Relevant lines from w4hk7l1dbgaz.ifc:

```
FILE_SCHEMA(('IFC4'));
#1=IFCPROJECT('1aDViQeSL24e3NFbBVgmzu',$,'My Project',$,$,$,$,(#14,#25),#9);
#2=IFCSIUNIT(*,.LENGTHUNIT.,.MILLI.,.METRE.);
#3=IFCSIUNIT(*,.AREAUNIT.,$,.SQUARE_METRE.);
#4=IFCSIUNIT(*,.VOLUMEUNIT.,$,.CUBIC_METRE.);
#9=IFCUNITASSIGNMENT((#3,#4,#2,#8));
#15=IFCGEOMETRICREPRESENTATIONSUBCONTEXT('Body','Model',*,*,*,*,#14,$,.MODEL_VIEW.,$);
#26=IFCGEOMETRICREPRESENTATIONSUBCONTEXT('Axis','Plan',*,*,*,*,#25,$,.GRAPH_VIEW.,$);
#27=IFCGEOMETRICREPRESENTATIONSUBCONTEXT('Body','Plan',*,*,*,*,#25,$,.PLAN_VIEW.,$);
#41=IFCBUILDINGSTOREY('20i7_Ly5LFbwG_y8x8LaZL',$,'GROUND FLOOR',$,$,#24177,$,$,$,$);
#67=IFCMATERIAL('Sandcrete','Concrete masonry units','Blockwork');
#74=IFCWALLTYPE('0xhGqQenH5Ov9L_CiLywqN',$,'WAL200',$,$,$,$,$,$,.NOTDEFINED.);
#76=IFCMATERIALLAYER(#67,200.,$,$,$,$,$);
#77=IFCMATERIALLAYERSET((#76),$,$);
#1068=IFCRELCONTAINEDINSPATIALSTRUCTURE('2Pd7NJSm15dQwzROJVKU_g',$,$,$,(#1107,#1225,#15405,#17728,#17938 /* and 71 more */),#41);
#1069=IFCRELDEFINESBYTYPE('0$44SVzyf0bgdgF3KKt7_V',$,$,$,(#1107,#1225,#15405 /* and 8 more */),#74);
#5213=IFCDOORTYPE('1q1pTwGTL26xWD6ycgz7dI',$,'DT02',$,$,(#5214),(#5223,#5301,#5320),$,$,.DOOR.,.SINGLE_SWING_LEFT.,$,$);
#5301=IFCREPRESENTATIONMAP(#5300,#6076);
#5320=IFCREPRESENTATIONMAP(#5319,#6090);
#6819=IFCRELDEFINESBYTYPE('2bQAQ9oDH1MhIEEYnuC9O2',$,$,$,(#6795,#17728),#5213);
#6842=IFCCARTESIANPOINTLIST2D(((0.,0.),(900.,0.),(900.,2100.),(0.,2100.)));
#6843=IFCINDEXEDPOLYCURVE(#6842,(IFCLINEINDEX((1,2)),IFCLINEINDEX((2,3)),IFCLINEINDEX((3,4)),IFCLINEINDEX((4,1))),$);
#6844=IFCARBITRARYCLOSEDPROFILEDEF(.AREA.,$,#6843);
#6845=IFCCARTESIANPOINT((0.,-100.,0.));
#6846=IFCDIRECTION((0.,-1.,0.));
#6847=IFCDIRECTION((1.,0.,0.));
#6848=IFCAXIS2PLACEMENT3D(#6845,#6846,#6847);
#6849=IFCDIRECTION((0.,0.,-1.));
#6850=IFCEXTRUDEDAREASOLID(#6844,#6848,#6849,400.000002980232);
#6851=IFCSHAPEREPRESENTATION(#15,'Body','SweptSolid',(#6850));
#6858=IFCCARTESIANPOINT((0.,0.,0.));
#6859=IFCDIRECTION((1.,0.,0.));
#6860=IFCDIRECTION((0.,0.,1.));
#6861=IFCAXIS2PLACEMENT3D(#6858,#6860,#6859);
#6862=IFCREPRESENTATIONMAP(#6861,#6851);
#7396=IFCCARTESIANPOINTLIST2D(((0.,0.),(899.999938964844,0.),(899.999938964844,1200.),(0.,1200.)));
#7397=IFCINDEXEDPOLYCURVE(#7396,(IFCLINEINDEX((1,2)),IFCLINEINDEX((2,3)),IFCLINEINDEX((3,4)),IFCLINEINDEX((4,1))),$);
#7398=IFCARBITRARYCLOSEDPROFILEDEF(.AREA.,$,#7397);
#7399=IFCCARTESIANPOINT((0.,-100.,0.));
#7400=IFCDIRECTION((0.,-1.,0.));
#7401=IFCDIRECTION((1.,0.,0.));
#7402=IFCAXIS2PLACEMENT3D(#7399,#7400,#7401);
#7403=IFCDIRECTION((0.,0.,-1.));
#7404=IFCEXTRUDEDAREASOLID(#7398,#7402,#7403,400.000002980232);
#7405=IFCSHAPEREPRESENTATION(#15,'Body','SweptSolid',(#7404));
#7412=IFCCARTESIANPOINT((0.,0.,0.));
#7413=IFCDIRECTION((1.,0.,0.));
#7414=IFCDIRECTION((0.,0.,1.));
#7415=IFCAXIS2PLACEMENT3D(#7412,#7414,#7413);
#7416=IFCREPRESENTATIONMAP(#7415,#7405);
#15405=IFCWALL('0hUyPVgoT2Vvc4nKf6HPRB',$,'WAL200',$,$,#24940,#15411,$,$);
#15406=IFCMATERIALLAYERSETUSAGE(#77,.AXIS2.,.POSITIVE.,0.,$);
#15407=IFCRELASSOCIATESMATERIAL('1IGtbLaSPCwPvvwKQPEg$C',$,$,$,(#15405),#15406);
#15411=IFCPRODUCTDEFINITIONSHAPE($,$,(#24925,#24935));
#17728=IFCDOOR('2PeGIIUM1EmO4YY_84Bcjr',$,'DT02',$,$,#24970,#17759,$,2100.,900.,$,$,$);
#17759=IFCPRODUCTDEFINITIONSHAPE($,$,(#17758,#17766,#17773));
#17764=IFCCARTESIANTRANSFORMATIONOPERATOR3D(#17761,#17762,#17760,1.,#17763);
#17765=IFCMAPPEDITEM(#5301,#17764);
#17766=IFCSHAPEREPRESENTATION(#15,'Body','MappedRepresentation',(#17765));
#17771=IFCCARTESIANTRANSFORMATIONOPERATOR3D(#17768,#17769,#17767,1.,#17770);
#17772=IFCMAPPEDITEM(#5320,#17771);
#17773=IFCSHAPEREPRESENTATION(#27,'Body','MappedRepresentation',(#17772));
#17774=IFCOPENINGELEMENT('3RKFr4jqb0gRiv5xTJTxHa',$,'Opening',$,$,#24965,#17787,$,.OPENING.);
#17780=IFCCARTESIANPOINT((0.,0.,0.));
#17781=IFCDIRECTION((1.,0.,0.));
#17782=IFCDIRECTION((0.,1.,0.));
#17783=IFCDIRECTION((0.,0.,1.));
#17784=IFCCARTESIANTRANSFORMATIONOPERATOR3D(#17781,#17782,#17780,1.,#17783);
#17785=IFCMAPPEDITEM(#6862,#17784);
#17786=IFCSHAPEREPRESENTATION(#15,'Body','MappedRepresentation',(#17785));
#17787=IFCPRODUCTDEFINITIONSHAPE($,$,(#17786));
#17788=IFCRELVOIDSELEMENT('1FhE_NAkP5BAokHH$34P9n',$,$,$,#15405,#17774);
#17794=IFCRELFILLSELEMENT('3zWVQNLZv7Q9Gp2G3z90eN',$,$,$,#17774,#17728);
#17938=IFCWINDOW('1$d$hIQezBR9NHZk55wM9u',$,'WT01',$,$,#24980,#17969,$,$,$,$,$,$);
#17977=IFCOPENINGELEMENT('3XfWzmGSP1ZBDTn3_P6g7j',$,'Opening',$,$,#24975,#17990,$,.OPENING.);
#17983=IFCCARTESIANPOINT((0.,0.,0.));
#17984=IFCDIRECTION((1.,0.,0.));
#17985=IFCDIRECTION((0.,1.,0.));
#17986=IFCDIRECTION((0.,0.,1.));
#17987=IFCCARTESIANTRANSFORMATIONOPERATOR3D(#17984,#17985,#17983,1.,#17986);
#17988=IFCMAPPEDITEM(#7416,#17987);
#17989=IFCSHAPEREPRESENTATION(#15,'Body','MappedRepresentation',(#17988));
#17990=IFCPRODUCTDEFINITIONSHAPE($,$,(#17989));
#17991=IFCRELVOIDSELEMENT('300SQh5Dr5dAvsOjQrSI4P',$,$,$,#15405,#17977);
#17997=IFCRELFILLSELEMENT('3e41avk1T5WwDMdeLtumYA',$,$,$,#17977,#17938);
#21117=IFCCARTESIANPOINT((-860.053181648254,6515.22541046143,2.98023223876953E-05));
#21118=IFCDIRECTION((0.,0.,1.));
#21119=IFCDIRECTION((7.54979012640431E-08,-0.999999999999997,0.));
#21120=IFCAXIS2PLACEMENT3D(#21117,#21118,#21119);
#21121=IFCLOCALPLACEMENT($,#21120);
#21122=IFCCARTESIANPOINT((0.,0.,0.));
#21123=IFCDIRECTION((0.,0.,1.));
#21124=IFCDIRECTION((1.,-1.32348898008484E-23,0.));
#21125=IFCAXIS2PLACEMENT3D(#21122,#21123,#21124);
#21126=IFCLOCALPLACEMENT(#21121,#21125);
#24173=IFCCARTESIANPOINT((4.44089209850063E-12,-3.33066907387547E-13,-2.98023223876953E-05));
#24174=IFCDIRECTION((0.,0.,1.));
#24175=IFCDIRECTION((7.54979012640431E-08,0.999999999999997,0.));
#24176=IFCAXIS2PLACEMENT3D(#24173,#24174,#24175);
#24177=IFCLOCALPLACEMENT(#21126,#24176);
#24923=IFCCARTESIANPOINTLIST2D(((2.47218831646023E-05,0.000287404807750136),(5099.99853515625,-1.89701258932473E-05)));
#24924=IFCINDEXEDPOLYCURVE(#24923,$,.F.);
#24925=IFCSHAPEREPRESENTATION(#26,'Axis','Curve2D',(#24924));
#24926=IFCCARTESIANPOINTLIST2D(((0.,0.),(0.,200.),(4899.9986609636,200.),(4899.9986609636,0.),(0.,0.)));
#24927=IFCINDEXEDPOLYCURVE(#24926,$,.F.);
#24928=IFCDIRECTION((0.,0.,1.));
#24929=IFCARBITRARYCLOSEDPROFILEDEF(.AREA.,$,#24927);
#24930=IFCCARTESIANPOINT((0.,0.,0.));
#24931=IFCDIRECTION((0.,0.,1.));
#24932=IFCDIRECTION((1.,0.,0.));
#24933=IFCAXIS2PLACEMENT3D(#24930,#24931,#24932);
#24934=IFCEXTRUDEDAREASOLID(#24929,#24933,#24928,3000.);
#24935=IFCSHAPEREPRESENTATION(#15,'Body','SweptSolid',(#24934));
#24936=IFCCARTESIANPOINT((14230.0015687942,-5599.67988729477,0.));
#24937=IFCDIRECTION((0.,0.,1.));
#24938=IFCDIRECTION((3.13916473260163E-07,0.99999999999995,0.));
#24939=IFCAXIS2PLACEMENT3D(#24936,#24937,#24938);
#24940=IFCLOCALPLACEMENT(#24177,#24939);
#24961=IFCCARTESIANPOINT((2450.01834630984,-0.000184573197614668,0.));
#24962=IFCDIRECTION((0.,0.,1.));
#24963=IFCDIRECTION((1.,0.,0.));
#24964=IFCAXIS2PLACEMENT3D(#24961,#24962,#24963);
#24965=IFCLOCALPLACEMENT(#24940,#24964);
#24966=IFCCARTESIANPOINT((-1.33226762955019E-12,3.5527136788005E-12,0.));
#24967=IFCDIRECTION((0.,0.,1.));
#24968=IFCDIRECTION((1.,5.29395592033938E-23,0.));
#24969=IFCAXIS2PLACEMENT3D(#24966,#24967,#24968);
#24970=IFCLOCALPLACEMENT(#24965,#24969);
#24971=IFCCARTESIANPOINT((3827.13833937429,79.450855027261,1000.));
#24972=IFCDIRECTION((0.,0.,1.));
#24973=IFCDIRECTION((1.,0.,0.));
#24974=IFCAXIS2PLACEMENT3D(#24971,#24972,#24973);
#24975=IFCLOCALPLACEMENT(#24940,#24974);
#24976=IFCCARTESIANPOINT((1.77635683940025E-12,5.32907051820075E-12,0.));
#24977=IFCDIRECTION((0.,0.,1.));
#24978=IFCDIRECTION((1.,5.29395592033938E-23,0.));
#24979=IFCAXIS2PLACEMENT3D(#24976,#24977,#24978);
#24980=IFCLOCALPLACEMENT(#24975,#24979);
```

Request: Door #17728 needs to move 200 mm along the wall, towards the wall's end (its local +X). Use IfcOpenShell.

```python
import ifcopenshell
import ifcopenshell.api.geometry
import ifcopenshell.util.placement
import ifcopenshell.util.unit

model = ifcopenshell.open("w4hk7l1dbgaz.ifc")
unit_scale = ifcopenshell.util.unit.calculate_unit_scale(model)

door = model.by_guid("2PeGIIUM1EmO4YY_84Bcjr")
opening = door.FillsVoids[0].RelatingOpeningElement
wall = opening.VoidsElements[0].RelatingBuildingElement

wall_matrix = ifcopenshell.util.placement.get_local_placement(wall.ObjectPlacement)
shift = wall_matrix[:3, 0] * 0.2 / unit_scale
before = ifcopenshell.util.placement.get_local_placement(door.ObjectPlacement)[:3, 3].copy()

# The door is placed relative to its opening, so it follows when the opening moves.
matrix = ifcopenshell.util.placement.get_local_placement(opening.ObjectPlacement)
matrix[:3, 3] += shift
ifcopenshell.api.geometry.edit_object_placement(
    model, product=opening, matrix=matrix, is_si=False, should_transform_children=True
)

after = ifcopenshell.util.placement.get_local_placement(door.ObjectPlacement)[:3, 3]
print("door moved by", (after - before).round(3) + 0.0)

model.write("w4hk7l1dbgaz_edited.ifc")
```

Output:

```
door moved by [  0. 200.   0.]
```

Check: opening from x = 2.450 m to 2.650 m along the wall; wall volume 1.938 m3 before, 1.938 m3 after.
